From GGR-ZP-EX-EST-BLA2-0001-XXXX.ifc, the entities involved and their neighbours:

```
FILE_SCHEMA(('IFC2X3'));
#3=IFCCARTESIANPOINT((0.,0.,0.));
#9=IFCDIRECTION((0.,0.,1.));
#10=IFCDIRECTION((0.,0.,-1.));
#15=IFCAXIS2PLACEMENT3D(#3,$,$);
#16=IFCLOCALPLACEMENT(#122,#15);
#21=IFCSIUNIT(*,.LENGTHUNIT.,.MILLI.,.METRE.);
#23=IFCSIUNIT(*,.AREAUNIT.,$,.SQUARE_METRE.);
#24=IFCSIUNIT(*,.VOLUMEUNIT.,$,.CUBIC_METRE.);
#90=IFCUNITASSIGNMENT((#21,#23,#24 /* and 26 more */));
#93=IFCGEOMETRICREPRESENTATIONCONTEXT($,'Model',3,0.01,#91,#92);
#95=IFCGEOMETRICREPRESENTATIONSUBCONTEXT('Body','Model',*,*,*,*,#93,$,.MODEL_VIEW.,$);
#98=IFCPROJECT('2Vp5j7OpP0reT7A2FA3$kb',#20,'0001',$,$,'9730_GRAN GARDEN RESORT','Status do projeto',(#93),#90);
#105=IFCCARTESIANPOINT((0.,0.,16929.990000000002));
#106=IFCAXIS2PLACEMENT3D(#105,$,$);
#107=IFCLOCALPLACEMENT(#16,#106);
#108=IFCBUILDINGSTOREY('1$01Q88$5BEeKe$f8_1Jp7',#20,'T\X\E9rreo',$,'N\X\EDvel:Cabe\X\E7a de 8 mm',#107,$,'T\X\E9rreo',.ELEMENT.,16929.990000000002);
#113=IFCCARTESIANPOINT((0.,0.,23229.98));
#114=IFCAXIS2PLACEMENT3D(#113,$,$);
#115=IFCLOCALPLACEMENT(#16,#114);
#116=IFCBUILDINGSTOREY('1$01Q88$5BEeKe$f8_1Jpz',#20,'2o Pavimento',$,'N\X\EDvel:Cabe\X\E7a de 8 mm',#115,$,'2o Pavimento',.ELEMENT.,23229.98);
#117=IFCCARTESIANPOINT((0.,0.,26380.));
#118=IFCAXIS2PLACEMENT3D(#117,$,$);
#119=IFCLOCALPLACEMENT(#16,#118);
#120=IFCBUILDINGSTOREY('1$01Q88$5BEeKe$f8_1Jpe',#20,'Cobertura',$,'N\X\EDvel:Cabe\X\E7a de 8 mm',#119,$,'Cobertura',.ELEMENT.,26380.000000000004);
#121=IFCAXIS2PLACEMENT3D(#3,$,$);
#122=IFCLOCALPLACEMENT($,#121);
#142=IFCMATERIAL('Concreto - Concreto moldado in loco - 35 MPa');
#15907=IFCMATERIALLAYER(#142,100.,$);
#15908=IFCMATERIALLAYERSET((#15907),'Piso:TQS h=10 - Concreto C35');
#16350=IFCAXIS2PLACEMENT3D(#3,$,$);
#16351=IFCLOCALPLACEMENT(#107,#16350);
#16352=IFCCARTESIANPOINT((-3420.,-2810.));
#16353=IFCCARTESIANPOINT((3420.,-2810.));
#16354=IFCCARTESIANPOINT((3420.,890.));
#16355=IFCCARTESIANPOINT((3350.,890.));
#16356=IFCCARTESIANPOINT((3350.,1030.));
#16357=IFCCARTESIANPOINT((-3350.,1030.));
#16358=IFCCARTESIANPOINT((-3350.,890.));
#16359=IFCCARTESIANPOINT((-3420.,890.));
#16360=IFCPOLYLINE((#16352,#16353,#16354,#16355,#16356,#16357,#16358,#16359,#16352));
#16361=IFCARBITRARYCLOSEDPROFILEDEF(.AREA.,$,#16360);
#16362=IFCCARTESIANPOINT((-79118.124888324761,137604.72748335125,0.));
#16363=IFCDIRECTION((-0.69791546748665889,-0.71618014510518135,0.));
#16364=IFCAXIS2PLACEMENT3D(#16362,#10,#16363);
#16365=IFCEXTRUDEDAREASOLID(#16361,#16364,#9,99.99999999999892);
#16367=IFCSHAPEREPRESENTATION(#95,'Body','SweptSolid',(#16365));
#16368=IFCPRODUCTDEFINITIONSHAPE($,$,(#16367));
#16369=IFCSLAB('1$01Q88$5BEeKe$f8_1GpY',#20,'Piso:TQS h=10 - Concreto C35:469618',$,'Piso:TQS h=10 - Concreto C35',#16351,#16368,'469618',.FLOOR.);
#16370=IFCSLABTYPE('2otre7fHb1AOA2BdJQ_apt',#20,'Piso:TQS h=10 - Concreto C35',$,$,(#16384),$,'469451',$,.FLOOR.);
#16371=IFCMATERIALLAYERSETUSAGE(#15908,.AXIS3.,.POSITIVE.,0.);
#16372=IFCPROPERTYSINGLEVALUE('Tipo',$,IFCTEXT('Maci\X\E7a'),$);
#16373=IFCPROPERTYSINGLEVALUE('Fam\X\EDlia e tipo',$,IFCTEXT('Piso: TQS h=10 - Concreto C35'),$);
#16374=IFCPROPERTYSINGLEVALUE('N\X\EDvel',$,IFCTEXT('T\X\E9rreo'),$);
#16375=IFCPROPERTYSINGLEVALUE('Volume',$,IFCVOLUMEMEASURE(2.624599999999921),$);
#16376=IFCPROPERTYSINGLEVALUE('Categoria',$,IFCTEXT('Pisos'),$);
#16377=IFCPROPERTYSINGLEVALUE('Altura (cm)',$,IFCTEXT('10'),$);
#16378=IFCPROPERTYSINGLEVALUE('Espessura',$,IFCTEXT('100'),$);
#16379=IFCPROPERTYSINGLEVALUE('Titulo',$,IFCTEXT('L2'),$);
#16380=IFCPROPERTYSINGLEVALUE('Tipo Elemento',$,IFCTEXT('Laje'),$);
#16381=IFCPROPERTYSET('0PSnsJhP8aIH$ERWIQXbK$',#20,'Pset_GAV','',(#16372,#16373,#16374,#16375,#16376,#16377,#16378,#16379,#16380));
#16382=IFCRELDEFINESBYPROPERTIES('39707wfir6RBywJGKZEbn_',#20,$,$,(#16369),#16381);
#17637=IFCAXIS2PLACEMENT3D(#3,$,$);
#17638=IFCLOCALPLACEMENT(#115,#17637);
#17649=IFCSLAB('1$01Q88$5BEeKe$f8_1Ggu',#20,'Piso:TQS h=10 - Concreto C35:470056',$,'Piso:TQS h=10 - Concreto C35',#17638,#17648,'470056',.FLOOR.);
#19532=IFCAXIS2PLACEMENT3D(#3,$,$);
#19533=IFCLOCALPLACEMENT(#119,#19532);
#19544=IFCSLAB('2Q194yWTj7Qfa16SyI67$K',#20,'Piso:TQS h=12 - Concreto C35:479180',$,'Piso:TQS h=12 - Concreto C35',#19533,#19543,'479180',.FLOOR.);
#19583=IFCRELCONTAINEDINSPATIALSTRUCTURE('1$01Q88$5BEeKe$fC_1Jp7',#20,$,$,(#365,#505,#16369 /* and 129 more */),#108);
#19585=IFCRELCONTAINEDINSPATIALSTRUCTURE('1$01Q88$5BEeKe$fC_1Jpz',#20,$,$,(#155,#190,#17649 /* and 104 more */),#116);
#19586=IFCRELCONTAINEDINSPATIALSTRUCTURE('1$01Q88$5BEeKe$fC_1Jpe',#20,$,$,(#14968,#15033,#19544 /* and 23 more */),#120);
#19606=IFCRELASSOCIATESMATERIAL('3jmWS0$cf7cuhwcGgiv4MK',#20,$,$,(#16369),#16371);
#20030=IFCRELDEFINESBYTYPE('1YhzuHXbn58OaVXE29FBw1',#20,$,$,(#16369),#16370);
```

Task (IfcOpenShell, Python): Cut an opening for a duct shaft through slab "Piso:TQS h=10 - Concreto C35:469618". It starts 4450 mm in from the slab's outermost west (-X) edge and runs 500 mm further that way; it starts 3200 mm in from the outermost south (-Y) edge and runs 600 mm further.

```python
import numpy as np
import ifcopenshell
import ifcopenshell.api.feature
import ifcopenshell.api.geometry
import ifcopenshell.api.pset
import ifcopenshell.api.root
import ifcopenshell.geom
import ifcopenshell.util.element
import ifcopenshell.util.placement
import ifcopenshell.util.representation
import ifcopenshell.util.shape
import ifcopenshell.util.unit

model = ifcopenshell.open("GGR-ZP-EX-EST-BLA2-0001-XXXX.ifc")
unit_scale = ifcopenshell.util.unit.calculate_unit_scale(model)
volume_scale = ifcopenshell.util.unit.calculate_unit_scale(model, "VOLUMEUNIT")
settings = ifcopenshell.geom.settings()


def volume(element):
    """Net volume in cubic metres, openings subtracted."""
    shape = ifcopenshell.geom.create_shape(settings, element)
    return ifcopenshell.util.shape.get_volume(shape.geometry)


slab = model.by_guid("1$01Q88$5BEeKe$f8_1GpY")
before = volume(slab)

# Extent in the slab's own axes, in metres. The edges named are its -X and -Y sides.
slab_shape = ifcopenshell.geom.create_shape(settings, slab)
vertices = ifcopenshell.util.shape.get_vertices(slab_shape.geometry)
x_min, y_min, bottom = vertices.min(axis=0)
top = vertices[:, 2].max()

opening = ifcopenshell.api.root.create_entity(model, ifc_class="IfcOpeningElement", name="Duct shaft opening")
context = ifcopenshell.util.representation.get_context(model, "Model", "Body", "MODEL_VIEW")
width, depth = 0.5, 0.6
outline = [(0.0, 0.0), (width, 0.0), (width, depth), (0.0, depth), (0.0, 0.0)]
# Overshoot both faces by 50 mm so the cut is clean.
shape = ifcopenshell.api.geometry.add_slab_representation(
    model, context=context, depth=top - bottom + 0.1, polyline=outline
)
ifcopenshell.api.geometry.assign_representation(model, product=opening, representation=shape)

matrix = ifcopenshell.util.placement.get_local_placement(slab.ObjectPlacement)
matrix[:, 3] = matrix @ np.append(np.array([x_min + 4.45, y_min + 3.2, bottom - 0.05]) / unit_scale, 1.0)
ifcopenshell.api.geometry.edit_object_placement(model, product=opening, matrix=matrix, is_si=False)
ifcopenshell.api.feature.add_feature(model, feature=opening, element=slab)

after = volume(slab)

# Update the slab's stored quantities.
pset = model.by_id(ifcopenshell.util.element.get_pset(slab, "Pset_GAV", should_inherit=False)["id"])
ifcopenshell.api.pset.edit_pset(model, pset=pset, properties={
    "Volume": model.create_entity("IfcVolumeMeasure", after / volume_scale),
})

print(f"slab volume {before:.3f} -> {after:.3f} m3")

model.write("GGR-ZP-EX-EST-BLA2-0001-XXXX-out.ifc")
```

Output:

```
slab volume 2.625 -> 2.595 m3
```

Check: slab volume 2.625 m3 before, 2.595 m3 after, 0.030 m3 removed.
